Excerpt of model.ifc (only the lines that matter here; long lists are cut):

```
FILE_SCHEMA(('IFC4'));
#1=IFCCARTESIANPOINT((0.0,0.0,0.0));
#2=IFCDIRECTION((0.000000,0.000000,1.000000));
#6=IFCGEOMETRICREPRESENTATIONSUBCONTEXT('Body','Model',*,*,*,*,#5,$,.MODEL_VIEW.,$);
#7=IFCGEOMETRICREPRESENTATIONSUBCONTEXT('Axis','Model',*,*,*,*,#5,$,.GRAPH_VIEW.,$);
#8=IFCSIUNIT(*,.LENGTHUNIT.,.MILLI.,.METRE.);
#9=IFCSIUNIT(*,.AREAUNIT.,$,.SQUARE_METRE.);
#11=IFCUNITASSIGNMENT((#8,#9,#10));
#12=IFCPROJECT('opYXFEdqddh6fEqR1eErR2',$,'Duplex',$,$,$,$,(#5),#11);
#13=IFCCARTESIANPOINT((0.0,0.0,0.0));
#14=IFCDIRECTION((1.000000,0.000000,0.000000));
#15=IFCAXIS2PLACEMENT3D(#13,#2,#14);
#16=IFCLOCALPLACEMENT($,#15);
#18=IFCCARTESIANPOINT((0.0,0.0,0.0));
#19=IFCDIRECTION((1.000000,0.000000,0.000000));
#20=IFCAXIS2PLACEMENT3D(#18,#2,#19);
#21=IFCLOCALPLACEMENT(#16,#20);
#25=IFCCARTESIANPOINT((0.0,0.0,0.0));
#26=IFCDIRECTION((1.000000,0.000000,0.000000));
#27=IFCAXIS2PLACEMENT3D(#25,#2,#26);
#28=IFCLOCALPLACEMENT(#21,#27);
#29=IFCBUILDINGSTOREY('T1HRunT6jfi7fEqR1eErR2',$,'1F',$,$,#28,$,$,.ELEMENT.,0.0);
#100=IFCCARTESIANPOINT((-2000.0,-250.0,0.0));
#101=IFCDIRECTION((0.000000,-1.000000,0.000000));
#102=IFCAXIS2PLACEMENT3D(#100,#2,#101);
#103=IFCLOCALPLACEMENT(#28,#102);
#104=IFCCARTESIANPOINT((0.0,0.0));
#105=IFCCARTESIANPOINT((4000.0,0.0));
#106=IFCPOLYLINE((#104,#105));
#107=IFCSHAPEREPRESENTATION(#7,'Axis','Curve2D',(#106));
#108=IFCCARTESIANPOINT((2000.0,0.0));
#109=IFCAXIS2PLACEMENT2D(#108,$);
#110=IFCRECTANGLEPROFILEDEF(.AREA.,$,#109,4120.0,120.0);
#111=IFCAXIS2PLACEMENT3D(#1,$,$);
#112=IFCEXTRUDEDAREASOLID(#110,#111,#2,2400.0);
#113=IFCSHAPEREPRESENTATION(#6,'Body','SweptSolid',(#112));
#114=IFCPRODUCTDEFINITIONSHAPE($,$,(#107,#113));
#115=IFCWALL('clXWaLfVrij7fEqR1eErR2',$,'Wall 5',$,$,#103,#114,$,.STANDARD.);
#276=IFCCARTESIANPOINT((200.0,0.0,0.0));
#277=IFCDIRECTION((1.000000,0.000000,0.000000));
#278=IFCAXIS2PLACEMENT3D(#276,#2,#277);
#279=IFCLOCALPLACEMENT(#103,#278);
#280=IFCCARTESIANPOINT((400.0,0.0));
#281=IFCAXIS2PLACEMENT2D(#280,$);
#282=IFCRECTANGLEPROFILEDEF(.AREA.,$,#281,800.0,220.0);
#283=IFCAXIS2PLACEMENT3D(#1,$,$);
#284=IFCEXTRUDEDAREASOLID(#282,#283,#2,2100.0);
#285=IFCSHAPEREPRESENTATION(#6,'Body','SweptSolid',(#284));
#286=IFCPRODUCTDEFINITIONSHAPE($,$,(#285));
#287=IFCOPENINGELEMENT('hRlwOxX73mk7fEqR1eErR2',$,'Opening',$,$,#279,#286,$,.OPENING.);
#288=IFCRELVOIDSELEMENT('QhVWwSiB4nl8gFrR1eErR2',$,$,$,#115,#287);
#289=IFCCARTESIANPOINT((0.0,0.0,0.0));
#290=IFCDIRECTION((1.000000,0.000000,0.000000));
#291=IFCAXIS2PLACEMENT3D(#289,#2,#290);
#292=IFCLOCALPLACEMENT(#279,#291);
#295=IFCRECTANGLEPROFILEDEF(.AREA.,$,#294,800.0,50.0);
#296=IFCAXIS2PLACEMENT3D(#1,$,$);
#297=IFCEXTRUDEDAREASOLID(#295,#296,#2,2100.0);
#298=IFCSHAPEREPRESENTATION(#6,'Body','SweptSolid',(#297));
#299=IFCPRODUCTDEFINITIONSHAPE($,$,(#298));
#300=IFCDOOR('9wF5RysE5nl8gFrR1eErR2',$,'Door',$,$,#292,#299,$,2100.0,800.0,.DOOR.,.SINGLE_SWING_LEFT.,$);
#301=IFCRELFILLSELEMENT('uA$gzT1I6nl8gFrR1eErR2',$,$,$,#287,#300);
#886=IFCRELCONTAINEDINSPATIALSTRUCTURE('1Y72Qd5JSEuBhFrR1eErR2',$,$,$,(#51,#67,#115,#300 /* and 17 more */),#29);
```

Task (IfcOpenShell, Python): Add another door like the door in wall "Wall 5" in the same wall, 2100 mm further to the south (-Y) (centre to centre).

```python
import ifcopenshell
import ifcopenshell.api.feature
import ifcopenshell.api.geometry
import ifcopenshell.api.root
import ifcopenshell.geom
import ifcopenshell.util.element
import ifcopenshell.util.placement
import ifcopenshell.util.shape

model = ifcopenshell.open("model.ifc")
settings = ifcopenshell.geom.settings()


def volume(element):
    """Net volume in cubic metres, openings subtracted."""
    shape = ifcopenshell.geom.create_shape(settings, element)
    return ifcopenshell.util.shape.get_volume(shape.geometry)


door = model.by_id(300)
opening = door.FillsVoids[0].RelatingOpeningElement
wall = opening.VoidsElements[0].RelatingBuildingElement
before = volume(wall)
shift = ifcopenshell.util.placement.get_local_placement(wall.ObjectPlacement)[:3, 0] * 2100.0

# copy_class copies the void relationship, type, container and properties, but no geometry.
new_opening = ifcopenshell.api.root.copy_class(model, product=opening)
new_opening.Representation = ifcopenshell.util.element.copy_deep(
    model, opening.Representation, exclude=["IfcGeometricRepresentationContext", "IfcRepresentationMap"]
)
new_door = ifcopenshell.api.root.copy_class(model, product=door)
new_door.Representation = ifcopenshell.util.element.copy_deep(
    model, door.Representation, exclude=["IfcGeometricRepresentationContext", "IfcRepresentationMap"]
)
ifcopenshell.api.feature.add_filling(model, opening=new_opening, element=new_door)

for old, new in ((opening, new_opening), (door, new_door)):
    matrix = ifcopenshell.util.placement.get_local_placement(old.ObjectPlacement)
    matrix[:3, 3] += shift
    ifcopenshell.api.geometry.edit_object_placement(model, product=new, matrix=matrix, is_si=False)

after = volume(wall)

print(f"wall volume {before:.3f} -> {after:.3f} m3")

model.write("model_rev.ifc")
```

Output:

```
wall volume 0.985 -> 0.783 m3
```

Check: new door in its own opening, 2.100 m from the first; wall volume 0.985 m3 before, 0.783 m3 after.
